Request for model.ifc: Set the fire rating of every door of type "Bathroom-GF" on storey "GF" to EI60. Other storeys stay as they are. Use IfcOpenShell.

First a look at what the model holds.

```python
import ifcopenshell
import ifcopenshell.util.element

model = ifcopenshell.open("model.ifc")
print(model.schema)
storey = next(s for s in model.by_type("IfcBuildingStorey") if s.Name == "GF")
doors = [e for e in ifcopenshell.util.element.get_decomposition(storey) if e.is_a("IfcDoor")]
seen = {}
for e in doors:
    element_type = ifcopenshell.util.element.get_type(e)
    key = (element_type.Name if element_type != e and element_type else None, ifcopenshell.util.element.get_pset(e, "Pset_DoorCommon", "FireRating"))
    seen[key] = seen.get(key, 0) + 1
for (name, value), count in sorted(seen.items(), key=str):
    print(count, "x", name, "|", value)
```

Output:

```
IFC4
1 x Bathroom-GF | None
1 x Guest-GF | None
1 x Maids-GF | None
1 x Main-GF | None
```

```python
import ifcopenshell
import ifcopenshell.api.pset
import ifcopenshell.util.element

model = ifcopenshell.open("model.ifc")

storey = next(s for s in model.by_type("IfcBuildingStorey") if s.Name == "GF")
doors = [e for e in ifcopenshell.util.element.get_decomposition(storey) if e.is_a("IfcDoor")]

count = 0
for e in doors:
    element_type = ifcopenshell.util.element.get_type(e)
    if element_type in (None, e) or element_type.Name != "Bathroom-GF":
        continue
    # add_pset returns the element's existing set when there is one.
    pset = ifcopenshell.api.pset.add_pset(model, product=e, name="Pset_DoorCommon")
    ifcopenshell.api.pset.edit_pset(model, pset=pset, properties={"FireRating": "EI60"})
    count += 1

print(count, "doors updated")

model.write("model-out.ifc")
```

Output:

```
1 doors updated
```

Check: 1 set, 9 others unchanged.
